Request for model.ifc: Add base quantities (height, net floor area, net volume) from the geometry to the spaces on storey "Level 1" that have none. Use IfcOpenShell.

First a look at what the model holds.

```python
import ifcopenshell
import ifcopenshell.util.element
import ifcopenshell.util.unit

model = ifcopenshell.open("model.ifc")
print(model.schema)
for unit_type in ("LENGTHUNIT", "AREAUNIT", "VOLUMEUNIT"):
    print(unit_type, ifcopenshell.util.unit.calculate_unit_scale(model, unit_type))
storey = next(s for s in model.by_type("IfcBuildingStorey") if s.Name == "Level 1")
spaces = [e for e in ifcopenshell.util.element.get_decomposition(storey) if e.is_a("IfcSpace")]
for e in sorted(spaces, key=lambda e: e.id()):
    print(e.id(), e.is_a(), e.Name, list(ifcopenshell.util.element.get_psets(e, qtos_only=True)), sep=" | ")
```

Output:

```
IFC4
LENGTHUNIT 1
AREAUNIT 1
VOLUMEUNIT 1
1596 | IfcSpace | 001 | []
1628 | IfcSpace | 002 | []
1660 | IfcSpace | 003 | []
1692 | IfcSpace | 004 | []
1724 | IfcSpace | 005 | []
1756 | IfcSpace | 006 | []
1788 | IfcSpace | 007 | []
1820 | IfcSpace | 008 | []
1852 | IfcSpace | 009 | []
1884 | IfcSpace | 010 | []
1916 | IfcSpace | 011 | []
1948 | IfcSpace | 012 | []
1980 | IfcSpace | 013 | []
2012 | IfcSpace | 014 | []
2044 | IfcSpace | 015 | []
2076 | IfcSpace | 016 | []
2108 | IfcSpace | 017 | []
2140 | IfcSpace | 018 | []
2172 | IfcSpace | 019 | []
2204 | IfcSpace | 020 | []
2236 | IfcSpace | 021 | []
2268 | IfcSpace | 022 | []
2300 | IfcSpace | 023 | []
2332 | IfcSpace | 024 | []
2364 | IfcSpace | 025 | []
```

```python
import ifcopenshell
import ifcopenshell.api.pset
import ifcopenshell.geom
import ifcopenshell.util.element
import ifcopenshell.util.shape
import ifcopenshell.util.unit

model = ifcopenshell.open("model.ifc")
unit_scale = ifcopenshell.util.unit.calculate_unit_scale(model)
area_scale = ifcopenshell.util.unit.calculate_unit_scale(model, "AREAUNIT")
volume_scale = ifcopenshell.util.unit.calculate_unit_scale(model, "VOLUMEUNIT")
settings = ifcopenshell.geom.settings()

storey = next(s for s in model.by_type("IfcBuildingStorey") if s.Name == "Level 1")
spaces = [e for e in ifcopenshell.util.element.get_decomposition(storey) if e.is_a("IfcSpace")]

for e in sorted(spaces, key=lambda e: e.id()):
    if ifcopenshell.util.element.get_psets(e, qtos_only=True, should_inherit=False):
        continue
    # Geometry comes back in metres, in the element's own axes.
    shape = ifcopenshell.geom.create_shape(settings, e)
    values = {
        "Height": ifcopenshell.util.shape.get_z(shape.geometry) / unit_scale,
        "NetFloorArea": ifcopenshell.util.shape.get_footprint_area(shape.geometry) / area_scale,
        "NetVolume": ifcopenshell.util.shape.get_volume(shape.geometry) / volume_scale,
    }
    qto = ifcopenshell.api.pset.add_qto(model, product=e, name="Qto_SpaceBaseQuantities")
    ifcopenshell.api.pset.edit_qto(model, qto=qto, properties=values)
    print(e.id(), {k: round(v, 3) for k, v in values.items()})

model.write("model_updated.ifc")
```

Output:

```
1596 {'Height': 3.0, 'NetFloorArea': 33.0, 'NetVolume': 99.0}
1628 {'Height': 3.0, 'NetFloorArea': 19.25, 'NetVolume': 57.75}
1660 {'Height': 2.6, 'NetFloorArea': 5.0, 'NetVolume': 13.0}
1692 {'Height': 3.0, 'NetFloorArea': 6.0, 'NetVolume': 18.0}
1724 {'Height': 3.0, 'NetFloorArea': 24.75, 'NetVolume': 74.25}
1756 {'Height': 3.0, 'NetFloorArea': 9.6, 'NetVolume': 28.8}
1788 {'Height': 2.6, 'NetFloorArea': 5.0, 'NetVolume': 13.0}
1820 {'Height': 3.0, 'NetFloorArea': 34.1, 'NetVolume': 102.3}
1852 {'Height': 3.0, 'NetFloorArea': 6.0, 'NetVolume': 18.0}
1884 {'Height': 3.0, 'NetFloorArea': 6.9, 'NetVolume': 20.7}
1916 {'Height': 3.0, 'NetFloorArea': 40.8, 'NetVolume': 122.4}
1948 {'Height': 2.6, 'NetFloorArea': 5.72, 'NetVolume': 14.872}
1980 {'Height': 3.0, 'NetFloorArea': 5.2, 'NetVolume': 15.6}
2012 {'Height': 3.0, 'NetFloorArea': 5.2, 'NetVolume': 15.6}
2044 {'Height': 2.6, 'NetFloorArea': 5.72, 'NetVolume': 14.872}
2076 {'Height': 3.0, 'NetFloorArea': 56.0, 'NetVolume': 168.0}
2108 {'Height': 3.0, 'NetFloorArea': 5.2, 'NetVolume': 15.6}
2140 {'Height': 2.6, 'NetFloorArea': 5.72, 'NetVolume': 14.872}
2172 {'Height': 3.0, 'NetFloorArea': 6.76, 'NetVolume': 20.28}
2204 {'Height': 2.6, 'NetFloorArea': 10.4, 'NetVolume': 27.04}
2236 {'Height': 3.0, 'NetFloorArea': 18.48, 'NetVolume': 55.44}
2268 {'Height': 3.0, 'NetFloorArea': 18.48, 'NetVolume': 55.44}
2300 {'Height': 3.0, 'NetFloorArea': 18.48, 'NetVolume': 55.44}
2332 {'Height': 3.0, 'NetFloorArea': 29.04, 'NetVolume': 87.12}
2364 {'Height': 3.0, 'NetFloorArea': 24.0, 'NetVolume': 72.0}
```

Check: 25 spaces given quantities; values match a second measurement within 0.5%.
